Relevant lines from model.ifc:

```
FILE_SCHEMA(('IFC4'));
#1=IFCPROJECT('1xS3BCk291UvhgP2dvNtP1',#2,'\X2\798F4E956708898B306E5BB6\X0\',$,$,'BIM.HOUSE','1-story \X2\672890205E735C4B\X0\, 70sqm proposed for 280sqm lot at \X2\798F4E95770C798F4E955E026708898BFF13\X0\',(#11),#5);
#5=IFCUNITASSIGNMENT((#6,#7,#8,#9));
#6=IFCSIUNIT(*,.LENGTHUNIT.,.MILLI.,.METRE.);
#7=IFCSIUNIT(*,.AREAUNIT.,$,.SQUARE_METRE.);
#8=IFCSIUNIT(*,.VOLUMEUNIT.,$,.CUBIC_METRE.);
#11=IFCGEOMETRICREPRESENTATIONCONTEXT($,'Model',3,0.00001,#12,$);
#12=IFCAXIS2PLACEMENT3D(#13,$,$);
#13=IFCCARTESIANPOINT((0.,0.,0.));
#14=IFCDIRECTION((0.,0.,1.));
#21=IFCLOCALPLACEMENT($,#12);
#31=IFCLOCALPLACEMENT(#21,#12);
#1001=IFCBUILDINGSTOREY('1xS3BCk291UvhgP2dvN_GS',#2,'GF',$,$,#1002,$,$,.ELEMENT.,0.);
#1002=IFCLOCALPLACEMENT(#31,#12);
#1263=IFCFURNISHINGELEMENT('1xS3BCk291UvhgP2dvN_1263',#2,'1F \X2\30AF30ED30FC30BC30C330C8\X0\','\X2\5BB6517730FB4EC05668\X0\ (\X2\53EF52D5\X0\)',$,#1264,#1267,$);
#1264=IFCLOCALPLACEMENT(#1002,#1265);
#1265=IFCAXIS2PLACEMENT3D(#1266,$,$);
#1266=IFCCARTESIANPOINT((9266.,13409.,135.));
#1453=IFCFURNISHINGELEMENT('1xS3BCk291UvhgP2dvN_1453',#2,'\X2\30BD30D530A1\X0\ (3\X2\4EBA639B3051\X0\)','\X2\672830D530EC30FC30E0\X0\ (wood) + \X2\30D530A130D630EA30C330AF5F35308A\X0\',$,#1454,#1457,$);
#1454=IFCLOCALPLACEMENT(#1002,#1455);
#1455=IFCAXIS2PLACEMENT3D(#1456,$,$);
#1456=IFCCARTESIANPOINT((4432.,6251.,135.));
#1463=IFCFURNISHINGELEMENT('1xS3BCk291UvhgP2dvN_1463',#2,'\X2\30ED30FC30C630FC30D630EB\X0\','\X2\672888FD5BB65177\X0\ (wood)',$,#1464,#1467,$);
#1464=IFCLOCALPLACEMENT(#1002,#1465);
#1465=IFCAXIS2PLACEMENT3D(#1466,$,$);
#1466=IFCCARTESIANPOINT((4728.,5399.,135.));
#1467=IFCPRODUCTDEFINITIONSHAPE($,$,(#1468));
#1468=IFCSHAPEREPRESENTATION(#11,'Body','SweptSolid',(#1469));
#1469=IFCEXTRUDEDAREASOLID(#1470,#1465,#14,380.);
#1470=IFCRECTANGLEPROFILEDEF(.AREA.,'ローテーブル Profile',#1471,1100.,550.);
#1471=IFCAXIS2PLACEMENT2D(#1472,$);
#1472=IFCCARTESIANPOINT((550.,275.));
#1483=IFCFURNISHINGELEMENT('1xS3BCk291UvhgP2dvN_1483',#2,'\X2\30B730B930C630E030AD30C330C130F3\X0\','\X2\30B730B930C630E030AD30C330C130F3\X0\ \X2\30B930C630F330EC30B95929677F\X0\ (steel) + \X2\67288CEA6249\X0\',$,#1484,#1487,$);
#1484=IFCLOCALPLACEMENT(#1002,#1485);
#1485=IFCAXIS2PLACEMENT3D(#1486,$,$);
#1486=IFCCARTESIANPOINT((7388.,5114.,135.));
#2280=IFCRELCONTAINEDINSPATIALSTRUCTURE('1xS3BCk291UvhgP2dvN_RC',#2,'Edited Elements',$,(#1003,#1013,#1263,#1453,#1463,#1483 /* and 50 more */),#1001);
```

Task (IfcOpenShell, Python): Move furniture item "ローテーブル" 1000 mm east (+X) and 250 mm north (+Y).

```python
import ifcopenshell
import ifcopenshell.api.geometry
import ifcopenshell.util.placement

model = ifcopenshell.open("model.ifc")

item = model.by_guid("1xS3BCk291UvhgP2dvN_1463")
matrix = ifcopenshell.util.placement.get_local_placement(item.ObjectPlacement)
matrix[0, 3] += 1000.0
matrix[1, 3] += 250.0
ifcopenshell.api.geometry.edit_object_placement(model, product=item, matrix=matrix, is_si=False)

print(ifcopenshell.util.placement.get_local_placement(item.ObjectPlacement).round(3) + 0.0)

model.write("model_edited.ifc")
```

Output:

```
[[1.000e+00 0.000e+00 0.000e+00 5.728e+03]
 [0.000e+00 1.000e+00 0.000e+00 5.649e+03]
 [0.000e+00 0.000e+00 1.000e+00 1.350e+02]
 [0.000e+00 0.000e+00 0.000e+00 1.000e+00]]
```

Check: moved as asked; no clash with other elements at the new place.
